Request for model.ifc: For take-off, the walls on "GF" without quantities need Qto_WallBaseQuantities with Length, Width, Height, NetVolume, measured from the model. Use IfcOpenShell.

First a look at what the model holds.

```python
import ifcopenshell
import ifcopenshell.util.element
import ifcopenshell.util.unit

model = ifcopenshell.open("model.ifc")
print(model.schema)
for unit_type in ("LENGTHUNIT", "AREAUNIT", "VOLUMEUNIT"):
    print(unit_type, ifcopenshell.util.unit.calculate_unit_scale(model, unit_type))
storey = next(s for s in model.by_type("IfcBuildingStorey") if s.Name == "GF")
walls = [e for e in ifcopenshell.util.element.get_decomposition(storey) if e.is_a("IfcWall")]
for e in sorted(walls, key=lambda e: e.id()):
    print(e.id(), e.is_a(), e.Name, list(ifcopenshell.util.element.get_psets(e, qtos_only=True)), sep=" | ")
```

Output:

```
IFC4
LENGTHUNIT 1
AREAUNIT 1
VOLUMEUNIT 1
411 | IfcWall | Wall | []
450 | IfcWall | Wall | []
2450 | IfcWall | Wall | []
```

```python
import ifcopenshell
import ifcopenshell.api.pset
import ifcopenshell.geom
import ifcopenshell.util.element
import ifcopenshell.util.shape
import ifcopenshell.util.unit

model = ifcopenshell.open("model.ifc")
unit_scale = ifcopenshell.util.unit.calculate_unit_scale(model)
volume_scale = ifcopenshell.util.unit.calculate_unit_scale(model, "VOLUMEUNIT")
settings = ifcopenshell.geom.settings()

storey = next(s for s in model.by_type("IfcBuildingStorey") if s.Name == "GF")
walls = [e for e in ifcopenshell.util.element.get_decomposition(storey) if e.is_a("IfcWall")]

for e in sorted(walls, key=lambda e: e.id()):
    if ifcopenshell.util.element.get_psets(e, qtos_only=True, should_inherit=False):
        continue
    # Geometry comes back in metres, in the element's own axes.
    shape = ifcopenshell.geom.create_shape(settings, e)
    values = {
        "Length": ifcopenshell.util.shape.get_x(shape.geometry) / unit_scale,
        "Width": ifcopenshell.util.shape.get_y(shape.geometry) / unit_scale,
        "Height": ifcopenshell.util.shape.get_z(shape.geometry) / unit_scale,
        "NetVolume": ifcopenshell.util.shape.get_volume(shape.geometry) / volume_scale,
    }
    qto = ifcopenshell.api.pset.add_qto(model, product=e, name="Qto_WallBaseQuantities")
    ifcopenshell.api.pset.edit_qto(model, qto=qto, properties=values)
    print(e.id(), {k: round(v, 3) for k, v in values.items()})

model.write("model_v2.ifc")
```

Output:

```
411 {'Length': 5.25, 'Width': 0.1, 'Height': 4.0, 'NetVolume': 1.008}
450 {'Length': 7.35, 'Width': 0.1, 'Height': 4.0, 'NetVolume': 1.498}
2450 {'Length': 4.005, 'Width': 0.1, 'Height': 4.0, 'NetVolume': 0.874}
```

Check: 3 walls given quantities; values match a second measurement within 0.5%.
